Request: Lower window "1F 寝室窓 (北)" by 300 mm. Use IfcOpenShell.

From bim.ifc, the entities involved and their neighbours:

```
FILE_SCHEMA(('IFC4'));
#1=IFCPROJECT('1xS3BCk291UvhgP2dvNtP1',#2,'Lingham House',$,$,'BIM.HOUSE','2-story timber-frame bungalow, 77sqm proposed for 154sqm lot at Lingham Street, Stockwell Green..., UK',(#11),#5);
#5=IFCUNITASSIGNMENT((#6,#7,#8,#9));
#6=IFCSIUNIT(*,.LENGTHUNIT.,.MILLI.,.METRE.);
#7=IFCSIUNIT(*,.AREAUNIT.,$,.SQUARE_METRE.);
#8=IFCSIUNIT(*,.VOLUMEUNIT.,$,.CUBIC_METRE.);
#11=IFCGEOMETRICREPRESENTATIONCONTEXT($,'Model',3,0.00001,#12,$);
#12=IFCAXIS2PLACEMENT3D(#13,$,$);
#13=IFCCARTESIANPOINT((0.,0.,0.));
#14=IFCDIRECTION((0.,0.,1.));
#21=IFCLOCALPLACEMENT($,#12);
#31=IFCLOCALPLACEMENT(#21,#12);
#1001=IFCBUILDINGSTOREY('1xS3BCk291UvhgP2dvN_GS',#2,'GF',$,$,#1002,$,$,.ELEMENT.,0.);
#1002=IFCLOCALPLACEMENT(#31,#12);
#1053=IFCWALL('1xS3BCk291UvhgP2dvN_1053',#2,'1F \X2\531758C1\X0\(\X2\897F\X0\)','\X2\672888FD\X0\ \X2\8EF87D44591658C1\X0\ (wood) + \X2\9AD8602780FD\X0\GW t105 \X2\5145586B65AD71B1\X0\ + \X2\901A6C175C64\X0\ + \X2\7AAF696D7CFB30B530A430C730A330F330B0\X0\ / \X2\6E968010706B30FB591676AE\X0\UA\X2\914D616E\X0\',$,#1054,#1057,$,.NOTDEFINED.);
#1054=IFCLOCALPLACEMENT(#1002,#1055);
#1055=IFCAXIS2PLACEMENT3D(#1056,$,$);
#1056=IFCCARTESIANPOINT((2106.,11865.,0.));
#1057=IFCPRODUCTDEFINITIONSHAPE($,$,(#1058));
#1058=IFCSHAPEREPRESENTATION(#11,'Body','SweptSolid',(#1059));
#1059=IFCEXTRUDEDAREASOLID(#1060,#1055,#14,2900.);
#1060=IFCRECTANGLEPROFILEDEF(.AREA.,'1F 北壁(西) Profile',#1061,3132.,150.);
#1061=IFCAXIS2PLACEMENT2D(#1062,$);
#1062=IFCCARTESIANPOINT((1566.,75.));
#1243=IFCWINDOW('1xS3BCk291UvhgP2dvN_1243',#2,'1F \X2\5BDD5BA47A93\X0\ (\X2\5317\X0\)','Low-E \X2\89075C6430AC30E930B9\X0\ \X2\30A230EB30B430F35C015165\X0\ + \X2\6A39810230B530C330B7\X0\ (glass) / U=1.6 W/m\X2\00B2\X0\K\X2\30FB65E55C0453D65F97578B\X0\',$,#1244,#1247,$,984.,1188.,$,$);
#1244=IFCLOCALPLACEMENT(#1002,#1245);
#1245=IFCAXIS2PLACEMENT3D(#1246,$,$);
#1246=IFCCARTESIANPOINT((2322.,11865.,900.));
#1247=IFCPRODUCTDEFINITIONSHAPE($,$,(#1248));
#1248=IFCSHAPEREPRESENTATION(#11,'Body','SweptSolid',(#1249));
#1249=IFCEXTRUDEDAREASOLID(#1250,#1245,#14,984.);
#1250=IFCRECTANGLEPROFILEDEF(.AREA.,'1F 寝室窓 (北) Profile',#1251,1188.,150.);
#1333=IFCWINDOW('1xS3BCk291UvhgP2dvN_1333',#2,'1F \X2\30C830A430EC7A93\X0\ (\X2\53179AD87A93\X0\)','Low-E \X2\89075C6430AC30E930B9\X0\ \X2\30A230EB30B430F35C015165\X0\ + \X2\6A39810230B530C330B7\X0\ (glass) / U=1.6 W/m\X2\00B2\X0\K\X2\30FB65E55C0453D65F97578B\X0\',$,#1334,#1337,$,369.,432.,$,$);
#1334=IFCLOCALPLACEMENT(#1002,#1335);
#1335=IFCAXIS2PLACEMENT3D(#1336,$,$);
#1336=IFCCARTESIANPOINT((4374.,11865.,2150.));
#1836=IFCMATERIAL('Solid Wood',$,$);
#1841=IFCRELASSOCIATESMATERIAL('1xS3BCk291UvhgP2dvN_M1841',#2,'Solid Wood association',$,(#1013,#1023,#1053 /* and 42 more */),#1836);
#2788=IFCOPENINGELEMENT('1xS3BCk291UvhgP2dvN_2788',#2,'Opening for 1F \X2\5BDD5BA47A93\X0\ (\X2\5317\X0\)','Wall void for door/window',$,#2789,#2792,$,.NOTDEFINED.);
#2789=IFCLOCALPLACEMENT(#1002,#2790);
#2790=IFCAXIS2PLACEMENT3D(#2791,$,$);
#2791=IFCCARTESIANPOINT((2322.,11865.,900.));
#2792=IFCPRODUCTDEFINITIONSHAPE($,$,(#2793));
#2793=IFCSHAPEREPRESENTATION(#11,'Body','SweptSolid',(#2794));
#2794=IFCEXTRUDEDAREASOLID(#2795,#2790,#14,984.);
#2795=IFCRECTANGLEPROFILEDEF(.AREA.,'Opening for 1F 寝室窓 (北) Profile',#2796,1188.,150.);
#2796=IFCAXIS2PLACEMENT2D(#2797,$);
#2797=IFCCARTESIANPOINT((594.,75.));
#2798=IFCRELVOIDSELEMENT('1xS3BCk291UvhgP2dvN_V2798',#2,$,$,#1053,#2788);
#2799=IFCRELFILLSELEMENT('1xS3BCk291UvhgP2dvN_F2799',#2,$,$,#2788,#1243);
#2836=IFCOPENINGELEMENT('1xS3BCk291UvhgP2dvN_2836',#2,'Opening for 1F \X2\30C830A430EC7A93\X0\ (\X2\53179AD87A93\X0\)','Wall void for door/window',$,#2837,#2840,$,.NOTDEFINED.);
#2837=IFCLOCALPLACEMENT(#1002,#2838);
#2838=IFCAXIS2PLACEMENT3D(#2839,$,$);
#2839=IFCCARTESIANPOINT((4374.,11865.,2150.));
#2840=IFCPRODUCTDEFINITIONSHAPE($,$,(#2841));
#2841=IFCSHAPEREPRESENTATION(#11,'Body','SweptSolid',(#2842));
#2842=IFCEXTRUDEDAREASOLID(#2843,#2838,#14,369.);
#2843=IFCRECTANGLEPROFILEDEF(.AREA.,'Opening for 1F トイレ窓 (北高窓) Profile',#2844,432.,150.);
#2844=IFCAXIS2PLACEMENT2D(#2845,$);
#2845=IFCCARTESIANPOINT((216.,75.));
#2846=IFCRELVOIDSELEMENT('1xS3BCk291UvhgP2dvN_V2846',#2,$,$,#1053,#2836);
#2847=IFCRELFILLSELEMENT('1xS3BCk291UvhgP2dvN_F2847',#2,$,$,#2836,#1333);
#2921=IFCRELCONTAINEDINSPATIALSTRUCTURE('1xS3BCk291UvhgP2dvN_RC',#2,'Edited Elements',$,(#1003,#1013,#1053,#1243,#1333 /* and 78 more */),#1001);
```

```python
import numpy as np
import ifcopenshell
import ifcopenshell.api.geometry
import ifcopenshell.util.placement
import ifcopenshell.util.unit

model = ifcopenshell.open("bim.ifc")
unit_scale = ifcopenshell.util.unit.calculate_unit_scale(model)

window = model.by_guid("1xS3BCk291UvhgP2dvN_1243")
opening = window.FillsVoids[0].RelatingOpeningElement
dz = -300.0

shift = np.array([0.0, 0.0, dz])
# The window is not placed relative to its opening, so move both.
for product in (opening, window):
    matrix = ifcopenshell.util.placement.get_local_placement(product.ObjectPlacement)
    matrix[:3, 3] += shift
    ifcopenshell.api.geometry.edit_object_placement(model, product=product, matrix=matrix, is_si=False)

print(f"moved by {dz * unit_scale:+.3f} m")

model.write("bim-out.ifc")
```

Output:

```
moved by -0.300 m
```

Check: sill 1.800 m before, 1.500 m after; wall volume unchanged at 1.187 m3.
